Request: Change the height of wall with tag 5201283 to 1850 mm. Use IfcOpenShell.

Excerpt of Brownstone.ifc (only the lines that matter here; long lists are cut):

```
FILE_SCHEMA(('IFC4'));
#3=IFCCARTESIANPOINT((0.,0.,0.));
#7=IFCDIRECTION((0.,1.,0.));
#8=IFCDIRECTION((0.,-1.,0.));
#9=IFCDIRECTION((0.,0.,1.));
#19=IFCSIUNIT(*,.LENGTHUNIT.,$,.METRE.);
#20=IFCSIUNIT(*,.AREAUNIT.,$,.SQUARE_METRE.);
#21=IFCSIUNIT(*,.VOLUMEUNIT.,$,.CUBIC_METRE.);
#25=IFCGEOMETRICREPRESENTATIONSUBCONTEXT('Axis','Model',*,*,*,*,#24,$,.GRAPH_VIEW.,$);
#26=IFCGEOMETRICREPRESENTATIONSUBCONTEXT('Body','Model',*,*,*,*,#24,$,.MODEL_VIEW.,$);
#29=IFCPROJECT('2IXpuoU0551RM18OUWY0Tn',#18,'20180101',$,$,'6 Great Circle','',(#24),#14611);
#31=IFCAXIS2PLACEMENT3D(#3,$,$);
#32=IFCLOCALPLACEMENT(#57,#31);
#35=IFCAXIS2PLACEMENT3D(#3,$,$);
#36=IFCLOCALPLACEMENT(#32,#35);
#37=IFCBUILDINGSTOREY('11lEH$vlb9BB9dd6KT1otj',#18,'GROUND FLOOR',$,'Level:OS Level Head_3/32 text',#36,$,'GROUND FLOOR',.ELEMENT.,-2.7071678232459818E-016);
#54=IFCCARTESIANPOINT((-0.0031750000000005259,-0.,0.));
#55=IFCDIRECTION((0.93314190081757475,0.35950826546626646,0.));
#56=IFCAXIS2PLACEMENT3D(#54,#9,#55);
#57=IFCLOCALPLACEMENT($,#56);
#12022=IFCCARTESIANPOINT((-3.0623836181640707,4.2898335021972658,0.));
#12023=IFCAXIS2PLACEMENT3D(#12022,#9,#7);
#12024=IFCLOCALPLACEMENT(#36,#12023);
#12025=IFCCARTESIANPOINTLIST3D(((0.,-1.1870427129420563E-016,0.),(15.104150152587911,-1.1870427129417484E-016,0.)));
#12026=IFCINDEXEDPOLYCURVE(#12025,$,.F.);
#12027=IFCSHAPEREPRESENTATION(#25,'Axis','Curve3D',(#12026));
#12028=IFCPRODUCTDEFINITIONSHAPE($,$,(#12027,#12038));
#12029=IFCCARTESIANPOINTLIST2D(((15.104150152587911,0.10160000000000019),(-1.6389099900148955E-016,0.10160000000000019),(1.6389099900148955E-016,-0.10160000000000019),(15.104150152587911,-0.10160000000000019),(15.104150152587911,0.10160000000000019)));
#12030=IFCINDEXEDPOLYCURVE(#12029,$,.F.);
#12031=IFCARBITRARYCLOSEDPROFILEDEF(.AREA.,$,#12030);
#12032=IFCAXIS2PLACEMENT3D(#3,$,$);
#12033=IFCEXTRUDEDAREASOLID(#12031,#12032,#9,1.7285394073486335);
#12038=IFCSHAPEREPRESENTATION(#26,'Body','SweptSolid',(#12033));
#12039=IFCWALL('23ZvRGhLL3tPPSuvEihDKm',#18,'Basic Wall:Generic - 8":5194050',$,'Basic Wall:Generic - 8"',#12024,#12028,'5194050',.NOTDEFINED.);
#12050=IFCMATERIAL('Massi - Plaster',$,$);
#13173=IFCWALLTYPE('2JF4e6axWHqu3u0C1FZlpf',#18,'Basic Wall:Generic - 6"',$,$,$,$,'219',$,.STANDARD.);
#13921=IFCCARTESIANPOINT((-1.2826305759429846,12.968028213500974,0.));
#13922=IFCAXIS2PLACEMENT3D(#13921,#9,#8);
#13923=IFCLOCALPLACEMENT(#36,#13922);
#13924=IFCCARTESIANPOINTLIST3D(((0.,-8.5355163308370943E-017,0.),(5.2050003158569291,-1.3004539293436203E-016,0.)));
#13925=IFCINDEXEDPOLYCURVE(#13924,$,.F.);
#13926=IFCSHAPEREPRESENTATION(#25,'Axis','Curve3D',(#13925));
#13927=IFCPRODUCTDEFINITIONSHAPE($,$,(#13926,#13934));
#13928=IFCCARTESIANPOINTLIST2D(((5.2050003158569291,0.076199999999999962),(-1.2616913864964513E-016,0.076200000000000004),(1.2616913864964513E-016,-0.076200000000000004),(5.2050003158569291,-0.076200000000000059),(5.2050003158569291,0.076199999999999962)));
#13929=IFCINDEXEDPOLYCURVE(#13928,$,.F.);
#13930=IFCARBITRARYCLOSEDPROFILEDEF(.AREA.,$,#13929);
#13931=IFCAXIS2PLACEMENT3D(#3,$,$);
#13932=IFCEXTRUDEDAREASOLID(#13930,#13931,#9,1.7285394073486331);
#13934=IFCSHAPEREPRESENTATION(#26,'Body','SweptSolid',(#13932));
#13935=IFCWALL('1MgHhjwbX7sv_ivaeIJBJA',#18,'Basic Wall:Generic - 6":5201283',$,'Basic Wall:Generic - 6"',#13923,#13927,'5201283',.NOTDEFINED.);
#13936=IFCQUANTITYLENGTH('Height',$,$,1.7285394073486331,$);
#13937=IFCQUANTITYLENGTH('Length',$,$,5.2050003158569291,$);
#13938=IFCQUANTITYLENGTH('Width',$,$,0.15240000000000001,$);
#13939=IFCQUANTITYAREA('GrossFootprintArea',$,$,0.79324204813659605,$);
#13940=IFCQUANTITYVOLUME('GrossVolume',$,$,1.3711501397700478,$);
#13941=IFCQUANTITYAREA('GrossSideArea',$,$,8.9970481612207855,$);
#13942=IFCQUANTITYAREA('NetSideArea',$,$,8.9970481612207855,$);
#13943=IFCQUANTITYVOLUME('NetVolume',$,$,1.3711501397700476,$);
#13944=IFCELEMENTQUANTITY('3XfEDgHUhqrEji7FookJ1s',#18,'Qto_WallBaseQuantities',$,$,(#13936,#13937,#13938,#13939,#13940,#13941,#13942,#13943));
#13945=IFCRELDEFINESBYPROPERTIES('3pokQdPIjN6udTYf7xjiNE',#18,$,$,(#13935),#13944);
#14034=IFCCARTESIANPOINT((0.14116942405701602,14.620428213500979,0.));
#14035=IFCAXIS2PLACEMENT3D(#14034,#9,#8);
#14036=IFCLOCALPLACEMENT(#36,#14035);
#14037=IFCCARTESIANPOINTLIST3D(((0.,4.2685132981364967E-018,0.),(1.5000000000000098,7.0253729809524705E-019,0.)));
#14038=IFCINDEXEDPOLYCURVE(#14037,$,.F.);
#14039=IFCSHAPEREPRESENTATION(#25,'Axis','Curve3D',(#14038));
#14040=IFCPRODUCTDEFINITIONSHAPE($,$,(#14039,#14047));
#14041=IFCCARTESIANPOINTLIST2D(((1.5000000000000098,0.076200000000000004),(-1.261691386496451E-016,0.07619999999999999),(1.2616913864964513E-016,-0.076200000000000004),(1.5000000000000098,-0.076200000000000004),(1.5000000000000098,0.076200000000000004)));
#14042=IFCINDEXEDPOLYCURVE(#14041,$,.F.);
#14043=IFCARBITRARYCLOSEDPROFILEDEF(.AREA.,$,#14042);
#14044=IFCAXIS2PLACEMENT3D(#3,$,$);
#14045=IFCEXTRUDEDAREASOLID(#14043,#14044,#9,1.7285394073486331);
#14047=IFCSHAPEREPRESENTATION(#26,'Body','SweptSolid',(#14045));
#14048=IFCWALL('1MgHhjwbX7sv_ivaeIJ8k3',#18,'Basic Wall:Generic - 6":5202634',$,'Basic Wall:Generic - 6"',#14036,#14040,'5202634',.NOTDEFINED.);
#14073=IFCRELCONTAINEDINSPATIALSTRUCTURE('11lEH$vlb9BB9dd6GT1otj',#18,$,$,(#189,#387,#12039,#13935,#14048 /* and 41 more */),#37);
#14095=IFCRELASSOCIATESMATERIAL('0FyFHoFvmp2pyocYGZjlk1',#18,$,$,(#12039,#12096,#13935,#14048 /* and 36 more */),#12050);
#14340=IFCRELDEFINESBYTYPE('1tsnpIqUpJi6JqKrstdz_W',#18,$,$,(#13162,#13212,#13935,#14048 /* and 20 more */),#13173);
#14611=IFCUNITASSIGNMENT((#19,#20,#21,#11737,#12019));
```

```python
import ifcopenshell
import ifcopenshell.api.pset
import ifcopenshell.geom
import ifcopenshell.util.element
import ifcopenshell.util.representation
import ifcopenshell.util.shape
import ifcopenshell.util.unit

model = ifcopenshell.open("Brownstone.ifc")
unit_scale = ifcopenshell.util.unit.calculate_unit_scale(model)
area_scale = ifcopenshell.util.unit.calculate_unit_scale(model, "AREAUNIT")
volume_scale = ifcopenshell.util.unit.calculate_unit_scale(model, "VOLUMEUNIT")
settings = ifcopenshell.geom.settings()


def volume(element):
    """Net volume in cubic metres, openings subtracted."""
    shape = ifcopenshell.geom.create_shape(settings, element)
    return ifcopenshell.util.shape.get_volume(shape.geometry)


wall = model.by_guid("1MgHhjwbX7sv_ivaeIJBJA")
before = volume(wall)

body = ifcopenshell.util.representation.get_representation(wall, "Model", "Body")
solid = body.Items[0]
old_height = solid.Depth
solid.Depth = 1.85
after = volume(wall)
thickness = 0.1524  # wall thickness in metres

# Update the stored height, areas and volumes.
qto = model.by_id(ifcopenshell.util.element.get_pset(wall, "Qto_WallBaseQuantities", should_inherit=False)["id"])
ifcopenshell.api.pset.edit_qto(model, qto=qto, properties={
    "Height": solid.Depth,
    "GrossVolume": ifcopenshell.util.element.get_pset(wall, "Qto_WallBaseQuantities", "GrossVolume") * solid.Depth / old_height,
    "GrossSideArea": ifcopenshell.util.element.get_pset(wall, "Qto_WallBaseQuantities", "GrossSideArea") * solid.Depth / old_height,
    "NetSideArea": after / thickness / area_scale,
    "NetVolume": after / volume_scale,
})

print(f"height {old_height:g} -> {solid.Depth:g}, volume {before:.3f} -> {after:.3f} m3")

model.write("Brownstone_updated.ifc")
```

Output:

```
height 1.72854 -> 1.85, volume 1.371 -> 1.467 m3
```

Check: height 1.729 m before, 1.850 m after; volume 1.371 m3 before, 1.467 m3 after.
